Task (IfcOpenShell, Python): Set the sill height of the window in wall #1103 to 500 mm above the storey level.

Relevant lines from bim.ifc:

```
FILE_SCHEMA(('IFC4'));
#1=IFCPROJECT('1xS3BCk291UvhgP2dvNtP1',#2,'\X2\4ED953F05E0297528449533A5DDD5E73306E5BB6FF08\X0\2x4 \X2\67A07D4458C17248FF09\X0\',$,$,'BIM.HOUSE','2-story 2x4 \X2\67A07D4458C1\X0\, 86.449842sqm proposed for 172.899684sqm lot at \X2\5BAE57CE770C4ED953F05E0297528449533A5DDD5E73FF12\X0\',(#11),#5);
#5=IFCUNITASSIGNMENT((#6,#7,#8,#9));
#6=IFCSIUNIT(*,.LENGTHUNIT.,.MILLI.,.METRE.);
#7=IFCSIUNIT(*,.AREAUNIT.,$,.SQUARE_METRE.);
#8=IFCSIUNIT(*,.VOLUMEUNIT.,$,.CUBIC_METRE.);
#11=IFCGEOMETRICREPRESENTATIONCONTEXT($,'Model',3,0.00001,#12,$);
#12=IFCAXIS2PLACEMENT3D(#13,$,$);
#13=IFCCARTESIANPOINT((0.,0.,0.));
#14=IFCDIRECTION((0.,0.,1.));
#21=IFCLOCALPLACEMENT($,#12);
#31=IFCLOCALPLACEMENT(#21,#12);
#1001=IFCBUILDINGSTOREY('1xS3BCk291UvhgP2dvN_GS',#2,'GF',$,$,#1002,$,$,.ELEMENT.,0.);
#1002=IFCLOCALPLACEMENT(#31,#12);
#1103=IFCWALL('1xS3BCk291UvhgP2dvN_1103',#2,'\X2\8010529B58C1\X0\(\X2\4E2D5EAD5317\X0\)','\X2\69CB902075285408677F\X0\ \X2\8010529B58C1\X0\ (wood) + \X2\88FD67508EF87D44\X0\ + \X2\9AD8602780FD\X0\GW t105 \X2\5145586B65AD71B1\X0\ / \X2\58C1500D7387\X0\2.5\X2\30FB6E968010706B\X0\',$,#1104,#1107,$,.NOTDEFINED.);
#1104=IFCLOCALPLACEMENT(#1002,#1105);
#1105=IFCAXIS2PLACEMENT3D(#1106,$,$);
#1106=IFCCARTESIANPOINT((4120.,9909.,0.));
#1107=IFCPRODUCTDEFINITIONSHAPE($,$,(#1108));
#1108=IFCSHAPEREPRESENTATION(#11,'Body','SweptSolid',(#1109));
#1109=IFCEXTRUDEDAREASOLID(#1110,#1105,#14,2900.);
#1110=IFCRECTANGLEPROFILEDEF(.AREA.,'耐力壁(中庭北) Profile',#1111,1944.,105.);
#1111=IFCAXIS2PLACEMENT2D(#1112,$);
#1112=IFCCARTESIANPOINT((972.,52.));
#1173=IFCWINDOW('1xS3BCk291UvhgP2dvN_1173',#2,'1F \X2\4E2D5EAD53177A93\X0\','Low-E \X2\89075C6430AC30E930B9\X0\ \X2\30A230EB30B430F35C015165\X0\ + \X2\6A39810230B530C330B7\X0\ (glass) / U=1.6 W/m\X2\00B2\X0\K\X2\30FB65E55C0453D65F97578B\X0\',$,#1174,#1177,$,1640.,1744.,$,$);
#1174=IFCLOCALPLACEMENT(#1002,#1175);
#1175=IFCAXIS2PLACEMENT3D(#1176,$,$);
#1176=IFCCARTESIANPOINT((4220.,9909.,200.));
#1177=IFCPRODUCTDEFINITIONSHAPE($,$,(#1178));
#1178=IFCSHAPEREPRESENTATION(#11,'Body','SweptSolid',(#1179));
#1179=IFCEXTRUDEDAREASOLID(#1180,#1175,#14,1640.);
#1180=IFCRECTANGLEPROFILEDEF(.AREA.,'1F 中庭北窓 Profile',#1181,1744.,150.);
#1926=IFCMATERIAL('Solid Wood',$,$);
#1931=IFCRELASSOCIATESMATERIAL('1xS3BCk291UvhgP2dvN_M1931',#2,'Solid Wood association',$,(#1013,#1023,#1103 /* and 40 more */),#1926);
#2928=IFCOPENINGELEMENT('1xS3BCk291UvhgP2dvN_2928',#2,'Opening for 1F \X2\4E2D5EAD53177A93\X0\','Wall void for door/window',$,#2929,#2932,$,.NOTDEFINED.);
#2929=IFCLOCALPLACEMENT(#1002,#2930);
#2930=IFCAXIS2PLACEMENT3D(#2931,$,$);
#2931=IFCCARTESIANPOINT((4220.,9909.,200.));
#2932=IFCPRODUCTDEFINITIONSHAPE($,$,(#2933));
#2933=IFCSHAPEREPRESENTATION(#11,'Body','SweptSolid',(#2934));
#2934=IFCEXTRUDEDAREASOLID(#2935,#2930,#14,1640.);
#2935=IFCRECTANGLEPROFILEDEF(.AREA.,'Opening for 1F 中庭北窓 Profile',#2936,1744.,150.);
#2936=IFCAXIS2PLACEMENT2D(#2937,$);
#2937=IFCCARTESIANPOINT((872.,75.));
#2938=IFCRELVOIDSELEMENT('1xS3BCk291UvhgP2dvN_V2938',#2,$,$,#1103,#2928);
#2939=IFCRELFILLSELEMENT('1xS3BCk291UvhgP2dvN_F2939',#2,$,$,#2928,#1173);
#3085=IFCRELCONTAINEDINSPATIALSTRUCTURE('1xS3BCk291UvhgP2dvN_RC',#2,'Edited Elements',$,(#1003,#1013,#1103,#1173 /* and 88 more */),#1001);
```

```python
import numpy as np
import ifcopenshell
import ifcopenshell.api.geometry
import ifcopenshell.geom
import ifcopenshell.util.element
import ifcopenshell.util.placement
import ifcopenshell.util.shape
import ifcopenshell.util.unit

model = ifcopenshell.open("bim.ifc")
unit_scale = ifcopenshell.util.unit.calculate_unit_scale(model)

window = model.by_guid("1xS3BCk291UvhgP2dvN_1173")
opening = window.FillsVoids[0].RelatingOpeningElement
storey = ifcopenshell.util.element.get_container(window, ifc_class="IfcBuildingStorey")
level = ifcopenshell.util.placement.get_local_placement(storey.ObjectPlacement)[2, 3]

# The opening's origin need not be at the sill, so measure its lowest point.
shape = ifcopenshell.geom.create_shape(ifcopenshell.geom.settings(), opening)
bottom = ifcopenshell.util.shape.get_shape_bottom_elevation(shape, shape.geometry) / unit_scale
dz = level + 0.5 / unit_scale - bottom

shift = np.array([0.0, 0.0, dz])
# The window is not placed relative to its opening, so move both.
for product in (opening, window):
    matrix = ifcopenshell.util.placement.get_local_placement(product.ObjectPlacement)
    matrix[:3, 3] += shift
    ifcopenshell.api.geometry.edit_object_placement(model, product=product, matrix=matrix, is_si=False)

print(f"moved by {dz * unit_scale:+.3f} m")

model.write("bim_updated.ifc")
```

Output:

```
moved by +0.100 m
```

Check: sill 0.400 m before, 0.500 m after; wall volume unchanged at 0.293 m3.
